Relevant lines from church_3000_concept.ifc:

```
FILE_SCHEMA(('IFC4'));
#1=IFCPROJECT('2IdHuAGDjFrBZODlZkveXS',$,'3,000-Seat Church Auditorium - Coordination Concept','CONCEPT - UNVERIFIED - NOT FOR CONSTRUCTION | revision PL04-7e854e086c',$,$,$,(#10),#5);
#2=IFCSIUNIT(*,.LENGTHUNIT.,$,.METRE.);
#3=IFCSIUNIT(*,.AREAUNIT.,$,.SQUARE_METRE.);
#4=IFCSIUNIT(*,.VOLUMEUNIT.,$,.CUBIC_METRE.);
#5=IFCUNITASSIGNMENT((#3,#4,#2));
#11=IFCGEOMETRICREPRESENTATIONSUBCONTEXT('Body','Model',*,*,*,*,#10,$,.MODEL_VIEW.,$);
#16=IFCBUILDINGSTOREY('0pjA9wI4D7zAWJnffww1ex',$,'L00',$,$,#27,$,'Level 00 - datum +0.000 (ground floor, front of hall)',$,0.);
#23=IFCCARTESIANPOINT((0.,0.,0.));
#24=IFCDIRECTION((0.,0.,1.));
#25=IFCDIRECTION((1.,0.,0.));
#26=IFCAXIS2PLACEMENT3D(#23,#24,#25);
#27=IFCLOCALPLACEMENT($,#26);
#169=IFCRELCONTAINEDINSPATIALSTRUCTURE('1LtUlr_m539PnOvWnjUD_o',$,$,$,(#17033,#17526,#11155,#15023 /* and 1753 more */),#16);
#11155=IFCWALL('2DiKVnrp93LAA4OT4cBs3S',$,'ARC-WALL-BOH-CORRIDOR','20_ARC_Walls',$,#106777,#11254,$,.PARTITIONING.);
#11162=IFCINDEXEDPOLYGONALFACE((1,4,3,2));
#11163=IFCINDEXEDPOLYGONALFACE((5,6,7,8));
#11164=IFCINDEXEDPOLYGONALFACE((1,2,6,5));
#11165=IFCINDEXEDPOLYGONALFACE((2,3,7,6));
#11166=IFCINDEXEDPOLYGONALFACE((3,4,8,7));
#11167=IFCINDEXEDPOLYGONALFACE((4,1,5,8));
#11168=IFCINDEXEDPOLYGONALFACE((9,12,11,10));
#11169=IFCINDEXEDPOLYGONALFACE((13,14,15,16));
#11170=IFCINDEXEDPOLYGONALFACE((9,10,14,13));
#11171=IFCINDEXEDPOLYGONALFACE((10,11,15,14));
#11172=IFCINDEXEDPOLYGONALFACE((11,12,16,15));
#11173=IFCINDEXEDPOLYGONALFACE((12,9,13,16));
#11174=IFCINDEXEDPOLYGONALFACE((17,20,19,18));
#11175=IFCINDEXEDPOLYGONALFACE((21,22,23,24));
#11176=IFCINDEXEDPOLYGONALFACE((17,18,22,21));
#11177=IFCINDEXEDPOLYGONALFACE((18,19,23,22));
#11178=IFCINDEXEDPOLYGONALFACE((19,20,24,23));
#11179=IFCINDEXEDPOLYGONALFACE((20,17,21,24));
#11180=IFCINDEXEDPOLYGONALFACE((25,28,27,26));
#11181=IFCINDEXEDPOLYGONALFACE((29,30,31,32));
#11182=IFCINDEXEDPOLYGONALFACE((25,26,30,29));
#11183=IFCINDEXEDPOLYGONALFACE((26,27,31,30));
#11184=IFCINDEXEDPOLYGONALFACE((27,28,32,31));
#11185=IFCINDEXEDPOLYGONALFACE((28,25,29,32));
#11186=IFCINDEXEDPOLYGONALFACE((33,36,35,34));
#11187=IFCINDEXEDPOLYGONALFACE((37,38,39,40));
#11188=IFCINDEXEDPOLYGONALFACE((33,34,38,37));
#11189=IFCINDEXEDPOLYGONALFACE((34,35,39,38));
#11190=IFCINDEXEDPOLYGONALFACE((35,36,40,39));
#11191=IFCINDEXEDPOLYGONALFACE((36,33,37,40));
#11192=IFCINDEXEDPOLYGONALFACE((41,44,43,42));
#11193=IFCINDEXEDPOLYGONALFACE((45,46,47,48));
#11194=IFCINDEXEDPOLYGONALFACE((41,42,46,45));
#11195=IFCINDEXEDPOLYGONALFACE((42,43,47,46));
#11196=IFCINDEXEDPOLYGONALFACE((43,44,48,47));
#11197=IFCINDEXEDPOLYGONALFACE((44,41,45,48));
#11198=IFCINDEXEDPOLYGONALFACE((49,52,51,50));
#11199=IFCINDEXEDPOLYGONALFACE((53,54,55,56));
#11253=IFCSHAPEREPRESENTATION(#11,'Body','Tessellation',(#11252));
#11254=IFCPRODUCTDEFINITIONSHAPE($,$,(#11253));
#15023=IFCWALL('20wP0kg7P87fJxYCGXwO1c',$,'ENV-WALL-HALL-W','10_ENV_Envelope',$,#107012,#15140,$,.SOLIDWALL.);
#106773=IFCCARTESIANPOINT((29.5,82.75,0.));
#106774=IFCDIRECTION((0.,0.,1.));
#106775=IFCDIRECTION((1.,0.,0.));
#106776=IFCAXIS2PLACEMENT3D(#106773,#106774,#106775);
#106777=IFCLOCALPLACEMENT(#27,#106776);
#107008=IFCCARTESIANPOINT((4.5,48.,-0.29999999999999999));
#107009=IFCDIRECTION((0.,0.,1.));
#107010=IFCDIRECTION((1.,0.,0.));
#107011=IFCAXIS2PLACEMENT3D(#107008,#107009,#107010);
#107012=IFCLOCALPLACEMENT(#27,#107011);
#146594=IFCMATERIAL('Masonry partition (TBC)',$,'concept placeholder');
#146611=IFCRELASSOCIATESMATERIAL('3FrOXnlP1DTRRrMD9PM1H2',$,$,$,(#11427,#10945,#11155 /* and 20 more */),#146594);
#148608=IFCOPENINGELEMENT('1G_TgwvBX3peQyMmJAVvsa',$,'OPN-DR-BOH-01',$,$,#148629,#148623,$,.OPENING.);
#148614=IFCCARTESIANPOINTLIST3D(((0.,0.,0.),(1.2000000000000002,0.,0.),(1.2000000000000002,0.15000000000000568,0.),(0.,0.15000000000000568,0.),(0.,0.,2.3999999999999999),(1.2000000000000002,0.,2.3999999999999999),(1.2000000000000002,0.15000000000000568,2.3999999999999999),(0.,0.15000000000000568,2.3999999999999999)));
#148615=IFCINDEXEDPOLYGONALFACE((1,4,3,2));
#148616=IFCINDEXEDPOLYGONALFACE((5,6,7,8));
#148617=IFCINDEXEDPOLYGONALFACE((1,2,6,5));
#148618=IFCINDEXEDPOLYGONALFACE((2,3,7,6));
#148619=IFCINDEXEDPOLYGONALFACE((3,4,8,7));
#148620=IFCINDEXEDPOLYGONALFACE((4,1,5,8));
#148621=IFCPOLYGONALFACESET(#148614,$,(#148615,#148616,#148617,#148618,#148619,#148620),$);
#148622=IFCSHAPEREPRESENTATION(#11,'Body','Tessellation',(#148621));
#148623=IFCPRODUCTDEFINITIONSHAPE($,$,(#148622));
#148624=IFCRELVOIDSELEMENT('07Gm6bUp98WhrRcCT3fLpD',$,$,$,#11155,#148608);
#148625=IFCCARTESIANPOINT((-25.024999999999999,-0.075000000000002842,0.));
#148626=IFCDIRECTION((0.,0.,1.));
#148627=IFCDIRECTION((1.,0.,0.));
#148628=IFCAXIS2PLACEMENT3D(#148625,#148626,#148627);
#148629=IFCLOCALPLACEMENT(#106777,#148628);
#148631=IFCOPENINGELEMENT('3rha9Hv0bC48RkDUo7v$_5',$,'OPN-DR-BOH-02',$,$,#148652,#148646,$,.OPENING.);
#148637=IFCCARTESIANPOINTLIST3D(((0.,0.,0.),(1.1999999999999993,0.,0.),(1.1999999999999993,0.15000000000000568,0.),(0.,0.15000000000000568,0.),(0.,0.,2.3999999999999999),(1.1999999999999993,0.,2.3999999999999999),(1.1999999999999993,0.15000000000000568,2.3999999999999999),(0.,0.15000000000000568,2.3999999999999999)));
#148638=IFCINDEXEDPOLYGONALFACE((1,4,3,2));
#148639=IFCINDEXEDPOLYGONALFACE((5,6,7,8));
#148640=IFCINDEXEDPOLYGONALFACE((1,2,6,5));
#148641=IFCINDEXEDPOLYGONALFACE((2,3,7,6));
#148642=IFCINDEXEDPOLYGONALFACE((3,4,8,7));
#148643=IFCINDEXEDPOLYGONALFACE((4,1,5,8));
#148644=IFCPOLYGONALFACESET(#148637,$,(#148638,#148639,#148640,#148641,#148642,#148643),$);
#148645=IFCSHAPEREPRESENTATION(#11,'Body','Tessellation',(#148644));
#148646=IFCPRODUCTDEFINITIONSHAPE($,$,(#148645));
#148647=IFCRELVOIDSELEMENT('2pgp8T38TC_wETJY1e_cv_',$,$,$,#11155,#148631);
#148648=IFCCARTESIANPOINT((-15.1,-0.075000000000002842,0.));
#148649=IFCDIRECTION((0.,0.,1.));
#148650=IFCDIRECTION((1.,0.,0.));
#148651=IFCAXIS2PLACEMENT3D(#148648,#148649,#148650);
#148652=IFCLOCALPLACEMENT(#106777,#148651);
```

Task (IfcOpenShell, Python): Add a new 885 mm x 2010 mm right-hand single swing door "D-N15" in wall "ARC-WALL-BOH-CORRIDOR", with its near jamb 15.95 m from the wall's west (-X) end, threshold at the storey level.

```python
import numpy as np
import ifcopenshell
import ifcopenshell.api.feature
import ifcopenshell.api.geometry
import ifcopenshell.api.root
import ifcopenshell.api.spatial
import ifcopenshell.geom
import ifcopenshell.util.element
import ifcopenshell.util.placement
import ifcopenshell.util.representation
import ifcopenshell.util.shape
import ifcopenshell.util.unit

model = ifcopenshell.open("church_3000_concept.ifc")
unit_scale = ifcopenshell.util.unit.calculate_unit_scale(model)
settings = ifcopenshell.geom.settings()


def volume(element):
    """Net volume in cubic metres, openings subtracted."""
    shape = ifcopenshell.geom.create_shape(settings, element)
    return ifcopenshell.util.shape.get_volume(shape.geometry)


wall = model.by_guid("2DiKVnrp93LAA4OT4cBs3S")
storey = ifcopenshell.util.element.get_container(wall, ifc_class="IfcBuildingStorey")
context = ifcopenshell.util.representation.get_context(model, "Model", "Body", "MODEL_VIEW")
before = volume(wall)

width, height, from_end, sill = 0.885, 2.01, 15.95, 0.0  # metres

# The wall runs along its own X axis, and the end named is its -X end.
wall_shape = ifcopenshell.geom.create_shape(settings, wall)
x, y, z = ifcopenshell.util.shape.get_vertices(wall_shape.geometry).T
start = x.min() + from_end
face, thickness = float(y.min()), float(y.max() - y.min())
wall_matrix = ifcopenshell.util.placement.get_local_placement(wall.ObjectPlacement)
level = ifcopenshell.util.placement.get_local_placement(storey.ObjectPlacement)[2, 3]


def in_wall(x, y):
    """Placement at x, y metres in the wall's axes, at sill height."""
    matrix = wall_matrix.copy()
    matrix[:, 3] = wall_matrix @ np.array([x / unit_scale, y / unit_scale, 0.0, 1.0])
    matrix[2, 3] = level + sill / unit_scale
    return matrix


# Opening: a box that overshoots both wall faces by 50 mm.
opening = ifcopenshell.api.root.create_entity(model, ifc_class="IfcOpeningElement", predefined_type="OPENING")
box = ifcopenshell.api.geometry.add_wall_representation(
    model, context=context, length=width, height=height, thickness=thickness + 0.1
)
ifcopenshell.api.geometry.assign_representation(model, product=opening, representation=box)
ifcopenshell.api.geometry.edit_object_placement(model, product=opening, matrix=in_wall(start, face - 0.05), is_si=False)
ifcopenshell.api.feature.add_feature(model, feature=opening, element=wall)

door = ifcopenshell.api.root.create_entity(model, ifc_class="IfcDoor", name="D-N15", predefined_type="DOOR")
door.OverallWidth, door.OverallHeight = width / unit_scale, height / unit_scale
door.OperationType = "SINGLE_SWING_RIGHT"
body = ifcopenshell.api.geometry.add_door_representation(
    model,
    context=context,
    overall_width=door.OverallWidth,
    overall_height=door.OverallHeight,
    operation_type="SINGLE_SWING_RIGHT",
    lining_properties={"LiningDepth": thickness / unit_scale, "ThresholdDepth": thickness / unit_scale},
)
ifcopenshell.api.geometry.assign_representation(model, product=door, representation=body)
ifcopenshell.api.spatial.assign_container(model, products=[door], relating_structure=storey)
ifcopenshell.api.feature.add_filling(model, opening=opening, element=door)

# The lining spans the wall, so the door starts at the wall face.
ifcopenshell.api.geometry.edit_object_placement(model, product=door, matrix=in_wall(start, face), is_si=False)

after = volume(wall)

print(f"wall volume {before:.3f} -> {after:.3f} m3")

model.write("church_3000_concept_edited.ifc")
```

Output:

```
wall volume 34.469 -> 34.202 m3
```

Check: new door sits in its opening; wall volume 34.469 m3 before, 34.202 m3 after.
